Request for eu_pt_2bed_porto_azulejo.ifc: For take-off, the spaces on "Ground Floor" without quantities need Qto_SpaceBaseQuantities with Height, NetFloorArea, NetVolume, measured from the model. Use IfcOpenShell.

First a look at what the model holds.

```python
import ifcopenshell
import ifcopenshell.util.element
import ifcopenshell.util.unit

model = ifcopenshell.open("eu_pt_2bed_porto_azulejo.ifc")
print(model.schema)
for unit_type in ("LENGTHUNIT", "AREAUNIT", "VOLUMEUNIT"):
    print(unit_type, ifcopenshell.util.unit.calculate_unit_scale(model, unit_type))
storey = next(s for s in model.by_type("IfcBuildingStorey") if s.Name == "Ground Floor")
spaces = [e for e in ifcopenshell.util.element.get_decomposition(storey) if e.is_a("IfcSpace")]
for e in sorted(spaces, key=lambda e: e.id()):
    print(e.id(), e.is_a(), e.Name, list(ifcopenshell.util.element.get_psets(e, qtos_only=True)), sep=" | ")
```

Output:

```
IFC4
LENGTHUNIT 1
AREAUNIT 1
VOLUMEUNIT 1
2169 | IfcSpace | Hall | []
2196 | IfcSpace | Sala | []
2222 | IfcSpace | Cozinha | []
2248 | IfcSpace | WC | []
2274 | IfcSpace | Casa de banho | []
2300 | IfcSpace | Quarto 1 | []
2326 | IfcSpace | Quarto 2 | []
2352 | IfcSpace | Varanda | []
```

```python
import ifcopenshell
import ifcopenshell.api.pset
import ifcopenshell.geom
import ifcopenshell.util.element
import ifcopenshell.util.shape
import ifcopenshell.util.unit

model = ifcopenshell.open("eu_pt_2bed_porto_azulejo.ifc")
unit_scale = ifcopenshell.util.unit.calculate_unit_scale(model)
area_scale = ifcopenshell.util.unit.calculate_unit_scale(model, "AREAUNIT")
volume_scale = ifcopenshell.util.unit.calculate_unit_scale(model, "VOLUMEUNIT")
settings = ifcopenshell.geom.settings()

storey = next(s for s in model.by_type("IfcBuildingStorey") if s.Name == "Ground Floor")
spaces = [e for e in ifcopenshell.util.element.get_decomposition(storey) if e.is_a("IfcSpace")]

for e in sorted(spaces, key=lambda e: e.id()):
    if ifcopenshell.util.element.get_psets(e, qtos_only=True, should_inherit=False):
        continue
    # Geometry comes back in metres, in the element's own axes.
    shape = ifcopenshell.geom.create_shape(settings, e)
    values = {
        "Height": ifcopenshell.util.shape.get_z(shape.geometry) / unit_scale,
        "NetFloorArea": ifcopenshell.util.shape.get_footprint_area(shape.geometry) / area_scale,
        "NetVolume": ifcopenshell.util.shape.get_volume(shape.geometry) / volume_scale,
    }
    qto = ifcopenshell.api.pset.add_qto(model, product=e, name="Qto_SpaceBaseQuantities")
    ifcopenshell.api.pset.edit_qto(model, qto=qto, properties=values)
    print(e.id(), {k: round(v, 3) for k, v in values.items()})

model.write("eu_pt_2bed_porto_azulejo_rev.ifc")
```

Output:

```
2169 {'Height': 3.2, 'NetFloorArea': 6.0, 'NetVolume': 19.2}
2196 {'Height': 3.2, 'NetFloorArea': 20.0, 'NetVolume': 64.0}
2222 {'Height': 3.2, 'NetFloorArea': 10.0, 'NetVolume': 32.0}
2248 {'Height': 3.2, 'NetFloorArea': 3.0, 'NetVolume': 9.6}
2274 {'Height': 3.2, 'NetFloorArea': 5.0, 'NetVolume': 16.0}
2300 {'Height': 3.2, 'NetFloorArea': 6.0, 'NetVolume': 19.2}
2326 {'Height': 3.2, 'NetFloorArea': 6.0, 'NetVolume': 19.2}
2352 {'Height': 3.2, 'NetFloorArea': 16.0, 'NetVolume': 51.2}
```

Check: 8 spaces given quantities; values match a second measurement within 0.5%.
